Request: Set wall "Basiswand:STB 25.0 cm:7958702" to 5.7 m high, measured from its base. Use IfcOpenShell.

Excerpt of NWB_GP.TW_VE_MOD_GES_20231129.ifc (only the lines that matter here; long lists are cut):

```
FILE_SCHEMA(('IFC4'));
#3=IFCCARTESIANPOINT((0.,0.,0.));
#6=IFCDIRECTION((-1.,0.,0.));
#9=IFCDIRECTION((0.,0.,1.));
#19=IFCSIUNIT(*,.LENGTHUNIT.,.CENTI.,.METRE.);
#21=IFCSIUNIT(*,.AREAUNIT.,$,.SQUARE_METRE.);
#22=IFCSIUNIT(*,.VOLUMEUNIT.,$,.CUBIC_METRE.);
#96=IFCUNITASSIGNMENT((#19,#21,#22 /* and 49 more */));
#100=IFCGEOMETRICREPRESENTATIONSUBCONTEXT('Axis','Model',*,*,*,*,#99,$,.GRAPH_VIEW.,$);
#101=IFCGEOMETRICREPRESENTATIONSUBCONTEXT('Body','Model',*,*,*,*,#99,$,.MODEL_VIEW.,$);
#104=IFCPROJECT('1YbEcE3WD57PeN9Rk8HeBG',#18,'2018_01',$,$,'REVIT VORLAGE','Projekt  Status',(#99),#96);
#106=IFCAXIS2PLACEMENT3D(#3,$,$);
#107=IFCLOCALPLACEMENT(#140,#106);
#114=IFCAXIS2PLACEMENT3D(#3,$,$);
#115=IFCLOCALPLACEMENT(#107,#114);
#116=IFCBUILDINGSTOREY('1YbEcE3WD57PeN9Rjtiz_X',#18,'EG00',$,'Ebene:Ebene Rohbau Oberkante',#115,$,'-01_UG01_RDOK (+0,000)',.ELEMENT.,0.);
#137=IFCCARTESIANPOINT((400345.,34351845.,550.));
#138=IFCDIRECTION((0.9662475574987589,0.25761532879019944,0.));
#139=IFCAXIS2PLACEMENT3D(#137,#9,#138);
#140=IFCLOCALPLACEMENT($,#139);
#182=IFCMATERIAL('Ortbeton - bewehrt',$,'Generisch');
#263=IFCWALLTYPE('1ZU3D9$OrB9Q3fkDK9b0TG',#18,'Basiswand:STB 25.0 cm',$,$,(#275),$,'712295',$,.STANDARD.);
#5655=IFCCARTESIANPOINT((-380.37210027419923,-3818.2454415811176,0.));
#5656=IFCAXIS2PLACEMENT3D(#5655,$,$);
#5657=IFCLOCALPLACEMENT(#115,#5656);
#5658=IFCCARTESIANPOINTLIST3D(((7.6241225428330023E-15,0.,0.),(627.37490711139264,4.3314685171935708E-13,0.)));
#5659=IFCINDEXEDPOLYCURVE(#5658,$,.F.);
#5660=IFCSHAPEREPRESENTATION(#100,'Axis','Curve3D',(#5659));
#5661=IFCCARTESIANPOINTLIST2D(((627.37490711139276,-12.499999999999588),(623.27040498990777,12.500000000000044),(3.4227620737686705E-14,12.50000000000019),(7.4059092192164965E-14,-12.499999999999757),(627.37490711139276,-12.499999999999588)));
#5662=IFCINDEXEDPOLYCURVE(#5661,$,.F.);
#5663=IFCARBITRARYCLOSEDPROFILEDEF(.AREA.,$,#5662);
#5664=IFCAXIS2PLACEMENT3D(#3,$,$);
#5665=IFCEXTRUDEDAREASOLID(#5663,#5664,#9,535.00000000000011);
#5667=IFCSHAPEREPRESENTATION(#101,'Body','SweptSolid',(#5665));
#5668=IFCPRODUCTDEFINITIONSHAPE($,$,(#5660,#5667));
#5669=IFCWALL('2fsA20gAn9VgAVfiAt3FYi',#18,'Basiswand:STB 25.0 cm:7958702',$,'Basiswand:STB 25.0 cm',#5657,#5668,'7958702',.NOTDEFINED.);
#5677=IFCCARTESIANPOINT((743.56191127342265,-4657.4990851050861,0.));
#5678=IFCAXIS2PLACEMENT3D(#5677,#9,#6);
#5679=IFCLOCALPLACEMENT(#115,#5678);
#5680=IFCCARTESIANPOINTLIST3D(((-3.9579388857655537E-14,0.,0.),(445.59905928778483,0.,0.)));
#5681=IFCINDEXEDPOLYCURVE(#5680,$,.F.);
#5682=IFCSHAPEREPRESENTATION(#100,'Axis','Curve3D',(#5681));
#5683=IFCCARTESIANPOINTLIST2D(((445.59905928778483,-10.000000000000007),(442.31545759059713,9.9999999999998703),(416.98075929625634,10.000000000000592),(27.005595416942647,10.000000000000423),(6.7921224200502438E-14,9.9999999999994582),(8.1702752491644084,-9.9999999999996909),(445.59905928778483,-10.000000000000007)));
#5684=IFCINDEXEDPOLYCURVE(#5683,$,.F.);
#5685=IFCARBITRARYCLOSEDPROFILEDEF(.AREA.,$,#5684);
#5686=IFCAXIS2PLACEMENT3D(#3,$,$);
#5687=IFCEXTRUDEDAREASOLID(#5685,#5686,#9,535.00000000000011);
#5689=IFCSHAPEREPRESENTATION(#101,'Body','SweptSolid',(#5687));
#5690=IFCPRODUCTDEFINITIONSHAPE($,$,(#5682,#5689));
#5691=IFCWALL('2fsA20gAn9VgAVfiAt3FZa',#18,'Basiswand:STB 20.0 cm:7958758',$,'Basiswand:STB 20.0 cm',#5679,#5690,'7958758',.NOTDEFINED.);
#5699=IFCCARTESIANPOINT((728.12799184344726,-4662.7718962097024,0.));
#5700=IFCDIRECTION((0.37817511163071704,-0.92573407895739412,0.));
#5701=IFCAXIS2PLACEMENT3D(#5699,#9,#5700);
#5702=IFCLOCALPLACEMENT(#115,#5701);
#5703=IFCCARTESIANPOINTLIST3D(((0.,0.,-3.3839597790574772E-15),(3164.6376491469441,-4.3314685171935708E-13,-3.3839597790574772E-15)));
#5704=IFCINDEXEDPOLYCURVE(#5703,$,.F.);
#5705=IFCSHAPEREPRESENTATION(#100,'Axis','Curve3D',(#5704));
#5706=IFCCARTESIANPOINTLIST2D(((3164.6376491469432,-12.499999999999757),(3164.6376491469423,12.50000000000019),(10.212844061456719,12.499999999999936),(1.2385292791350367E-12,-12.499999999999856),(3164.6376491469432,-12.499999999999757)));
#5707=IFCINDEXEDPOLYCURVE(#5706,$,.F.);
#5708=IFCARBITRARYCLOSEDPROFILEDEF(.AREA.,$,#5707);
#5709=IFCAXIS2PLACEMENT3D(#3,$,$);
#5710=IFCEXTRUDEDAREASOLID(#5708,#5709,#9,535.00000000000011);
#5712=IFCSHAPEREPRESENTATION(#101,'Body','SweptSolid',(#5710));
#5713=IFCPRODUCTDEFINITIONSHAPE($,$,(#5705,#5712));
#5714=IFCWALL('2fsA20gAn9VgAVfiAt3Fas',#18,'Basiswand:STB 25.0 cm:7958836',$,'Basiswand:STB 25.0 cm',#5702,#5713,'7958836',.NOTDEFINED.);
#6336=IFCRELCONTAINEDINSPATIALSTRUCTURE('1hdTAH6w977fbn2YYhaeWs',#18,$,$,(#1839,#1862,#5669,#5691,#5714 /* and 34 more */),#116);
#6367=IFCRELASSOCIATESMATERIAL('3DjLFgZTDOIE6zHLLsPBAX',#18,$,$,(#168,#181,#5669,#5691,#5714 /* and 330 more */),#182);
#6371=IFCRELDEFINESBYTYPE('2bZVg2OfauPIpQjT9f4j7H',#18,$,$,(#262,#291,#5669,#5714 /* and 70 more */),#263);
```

```python
import ifcopenshell
import ifcopenshell.geom
import ifcopenshell.util.representation
import ifcopenshell.util.shape
import ifcopenshell.util.unit

model = ifcopenshell.open("NWB_GP.TW_VE_MOD_GES_20231129.ifc")
unit_scale = ifcopenshell.util.unit.calculate_unit_scale(model)
settings = ifcopenshell.geom.settings()


def volume(element):
    """Net volume in cubic metres, openings subtracted."""
    shape = ifcopenshell.geom.create_shape(settings, element)
    return ifcopenshell.util.shape.get_volume(shape.geometry)


wall = model.by_id(5669)
before = volume(wall)

body = ifcopenshell.util.representation.get_representation(wall, "Model", "Body")
solid = body.Items[0]
old_height = solid.Depth
solid.Depth = 5.7 / unit_scale
after = volume(wall)

print(f"height {old_height:g} -> {solid.Depth:g}, volume {before:.3f} -> {after:.3f} m3")

model.write("NWB_GP.TW_VE_MOD_GES_20231129_v2.ifc")
```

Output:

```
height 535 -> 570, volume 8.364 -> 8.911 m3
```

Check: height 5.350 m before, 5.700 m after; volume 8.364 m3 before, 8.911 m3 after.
